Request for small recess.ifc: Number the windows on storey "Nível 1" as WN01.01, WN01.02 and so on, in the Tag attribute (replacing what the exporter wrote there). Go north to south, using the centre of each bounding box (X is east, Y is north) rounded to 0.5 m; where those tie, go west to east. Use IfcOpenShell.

First a look at what the model holds.

```python
import ifcopenshell
import ifcopenshell.util.element
import ifcopenshell.util.placement

model = ifcopenshell.open("small recess.ifc")
print(model.schema)
storey = next(s for s in model.by_type("IfcBuildingStorey") if s.Name == "Nível 1")
windows = [e for e in ifcopenshell.util.element.get_decomposition(storey) if e.is_a("IfcWindow")]
for e in sorted(windows, key=lambda e: e.id()):
    origin = ifcopenshell.util.placement.get_local_placement(e.ObjectPlacement)[:3, 3]
    print(e.id(), e.Tag, e.Name, origin.round(2) + 0.0, sep=" | ")
```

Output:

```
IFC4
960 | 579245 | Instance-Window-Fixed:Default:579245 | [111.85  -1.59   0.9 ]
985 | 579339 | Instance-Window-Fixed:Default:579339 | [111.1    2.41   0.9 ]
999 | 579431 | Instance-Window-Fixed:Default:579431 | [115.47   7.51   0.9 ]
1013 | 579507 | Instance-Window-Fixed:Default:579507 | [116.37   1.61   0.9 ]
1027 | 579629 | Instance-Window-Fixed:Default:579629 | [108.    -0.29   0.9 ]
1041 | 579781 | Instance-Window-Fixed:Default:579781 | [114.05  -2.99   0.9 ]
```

```python
import ifcopenshell
import ifcopenshell.geom
import ifcopenshell.util.element
import ifcopenshell.util.shape

model = ifcopenshell.open("small recess.ifc")
settings = ifcopenshell.geom.settings()
settings.set("use-world-coords", True)


def centre(element):
    shape = ifcopenshell.geom.create_shape(settings, element)
    return ifcopenshell.util.shape.get_bbox_centroid(shape.geometry)


storey = next(s for s in model.by_type("IfcBuildingStorey") if s.Name == "Nível 1")
windows = [e for e in ifcopenshell.util.element.get_decomposition(storey) if e.is_a("IfcWindow")]

# Insertion points can sit at a corner or the storey origin, so sort by the geometry (in metres).
centres = {e: centre(e) for e in windows}
windows.sort(key=lambda e: (-round(centres[e][1] / 0.5), centres[e][0]))

for i, e in enumerate(windows, start=1):
    number = f"WN01.{i:02d}"
    e.Tag = number
    print(e.id(), number)

model.write("small recess_v2.ifc")
```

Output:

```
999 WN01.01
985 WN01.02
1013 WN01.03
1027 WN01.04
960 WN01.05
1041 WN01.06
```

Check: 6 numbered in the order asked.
